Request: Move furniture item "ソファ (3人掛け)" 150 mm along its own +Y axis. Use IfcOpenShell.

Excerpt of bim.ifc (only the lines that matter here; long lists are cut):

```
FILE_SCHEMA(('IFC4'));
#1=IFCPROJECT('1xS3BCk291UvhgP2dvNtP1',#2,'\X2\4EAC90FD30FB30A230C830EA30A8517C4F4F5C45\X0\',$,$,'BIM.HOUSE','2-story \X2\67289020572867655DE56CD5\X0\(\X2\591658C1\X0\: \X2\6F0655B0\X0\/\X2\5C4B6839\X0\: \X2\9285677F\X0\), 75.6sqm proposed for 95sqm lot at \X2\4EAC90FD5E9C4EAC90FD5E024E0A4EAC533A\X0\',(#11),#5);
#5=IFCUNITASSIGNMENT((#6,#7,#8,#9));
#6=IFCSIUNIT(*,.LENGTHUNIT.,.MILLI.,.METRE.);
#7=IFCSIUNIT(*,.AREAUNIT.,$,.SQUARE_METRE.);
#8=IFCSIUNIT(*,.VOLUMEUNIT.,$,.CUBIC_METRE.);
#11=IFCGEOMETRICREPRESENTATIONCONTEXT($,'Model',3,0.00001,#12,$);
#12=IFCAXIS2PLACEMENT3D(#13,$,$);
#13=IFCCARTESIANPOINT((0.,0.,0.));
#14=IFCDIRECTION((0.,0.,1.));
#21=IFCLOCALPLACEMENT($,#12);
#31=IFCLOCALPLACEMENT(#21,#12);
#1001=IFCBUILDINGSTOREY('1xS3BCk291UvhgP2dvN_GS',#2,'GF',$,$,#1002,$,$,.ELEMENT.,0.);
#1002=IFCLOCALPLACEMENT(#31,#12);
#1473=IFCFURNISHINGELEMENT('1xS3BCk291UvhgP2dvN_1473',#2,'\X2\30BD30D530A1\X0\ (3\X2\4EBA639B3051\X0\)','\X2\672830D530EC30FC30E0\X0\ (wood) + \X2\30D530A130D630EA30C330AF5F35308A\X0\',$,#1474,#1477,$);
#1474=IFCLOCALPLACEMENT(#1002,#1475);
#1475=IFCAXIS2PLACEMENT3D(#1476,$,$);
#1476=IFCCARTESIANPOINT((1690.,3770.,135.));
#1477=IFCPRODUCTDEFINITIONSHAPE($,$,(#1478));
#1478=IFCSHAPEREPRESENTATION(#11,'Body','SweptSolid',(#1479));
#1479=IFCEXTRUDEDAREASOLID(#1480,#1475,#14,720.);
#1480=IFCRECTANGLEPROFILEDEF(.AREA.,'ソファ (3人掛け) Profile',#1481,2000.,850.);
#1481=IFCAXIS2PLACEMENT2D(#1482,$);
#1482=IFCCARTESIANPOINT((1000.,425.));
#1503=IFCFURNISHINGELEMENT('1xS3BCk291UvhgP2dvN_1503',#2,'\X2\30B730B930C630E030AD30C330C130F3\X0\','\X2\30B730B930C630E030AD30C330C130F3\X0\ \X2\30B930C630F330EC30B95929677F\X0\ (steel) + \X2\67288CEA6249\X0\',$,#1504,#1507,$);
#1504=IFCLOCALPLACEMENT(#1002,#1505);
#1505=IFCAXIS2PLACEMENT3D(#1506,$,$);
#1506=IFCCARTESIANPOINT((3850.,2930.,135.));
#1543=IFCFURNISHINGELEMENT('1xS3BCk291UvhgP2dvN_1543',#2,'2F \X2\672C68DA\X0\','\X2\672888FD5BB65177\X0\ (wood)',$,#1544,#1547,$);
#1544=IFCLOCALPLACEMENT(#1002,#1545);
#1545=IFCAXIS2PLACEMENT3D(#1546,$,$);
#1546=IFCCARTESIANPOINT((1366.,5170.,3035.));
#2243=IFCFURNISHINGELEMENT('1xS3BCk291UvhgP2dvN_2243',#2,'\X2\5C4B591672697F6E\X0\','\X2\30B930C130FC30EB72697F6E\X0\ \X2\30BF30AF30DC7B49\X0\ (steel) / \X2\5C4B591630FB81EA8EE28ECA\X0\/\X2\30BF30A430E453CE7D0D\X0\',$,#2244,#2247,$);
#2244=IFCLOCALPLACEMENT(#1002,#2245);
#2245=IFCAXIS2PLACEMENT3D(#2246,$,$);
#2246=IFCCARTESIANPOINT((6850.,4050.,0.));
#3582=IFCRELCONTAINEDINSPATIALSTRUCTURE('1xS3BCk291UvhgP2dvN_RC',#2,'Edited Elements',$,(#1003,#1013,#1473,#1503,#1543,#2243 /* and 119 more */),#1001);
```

```python
import ifcopenshell
import ifcopenshell.api.geometry
import ifcopenshell.util.placement

model = ifcopenshell.open("bim.ifc")

item = model.by_guid("1xS3BCk291UvhgP2dvN_1473")
matrix = ifcopenshell.util.placement.get_local_placement(item.ObjectPlacement)
matrix[:3, 3] += matrix[:3, 1] * 150.0
ifcopenshell.api.geometry.edit_object_placement(model, product=item, matrix=matrix, is_si=False)

print(ifcopenshell.util.placement.get_local_placement(item.ObjectPlacement).round(3) + 0.0)

model.write("bim_v2.ifc")
```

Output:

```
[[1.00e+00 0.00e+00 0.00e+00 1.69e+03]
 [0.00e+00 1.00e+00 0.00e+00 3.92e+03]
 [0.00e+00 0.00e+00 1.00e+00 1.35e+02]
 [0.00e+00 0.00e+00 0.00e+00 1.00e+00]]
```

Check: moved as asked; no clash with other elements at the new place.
